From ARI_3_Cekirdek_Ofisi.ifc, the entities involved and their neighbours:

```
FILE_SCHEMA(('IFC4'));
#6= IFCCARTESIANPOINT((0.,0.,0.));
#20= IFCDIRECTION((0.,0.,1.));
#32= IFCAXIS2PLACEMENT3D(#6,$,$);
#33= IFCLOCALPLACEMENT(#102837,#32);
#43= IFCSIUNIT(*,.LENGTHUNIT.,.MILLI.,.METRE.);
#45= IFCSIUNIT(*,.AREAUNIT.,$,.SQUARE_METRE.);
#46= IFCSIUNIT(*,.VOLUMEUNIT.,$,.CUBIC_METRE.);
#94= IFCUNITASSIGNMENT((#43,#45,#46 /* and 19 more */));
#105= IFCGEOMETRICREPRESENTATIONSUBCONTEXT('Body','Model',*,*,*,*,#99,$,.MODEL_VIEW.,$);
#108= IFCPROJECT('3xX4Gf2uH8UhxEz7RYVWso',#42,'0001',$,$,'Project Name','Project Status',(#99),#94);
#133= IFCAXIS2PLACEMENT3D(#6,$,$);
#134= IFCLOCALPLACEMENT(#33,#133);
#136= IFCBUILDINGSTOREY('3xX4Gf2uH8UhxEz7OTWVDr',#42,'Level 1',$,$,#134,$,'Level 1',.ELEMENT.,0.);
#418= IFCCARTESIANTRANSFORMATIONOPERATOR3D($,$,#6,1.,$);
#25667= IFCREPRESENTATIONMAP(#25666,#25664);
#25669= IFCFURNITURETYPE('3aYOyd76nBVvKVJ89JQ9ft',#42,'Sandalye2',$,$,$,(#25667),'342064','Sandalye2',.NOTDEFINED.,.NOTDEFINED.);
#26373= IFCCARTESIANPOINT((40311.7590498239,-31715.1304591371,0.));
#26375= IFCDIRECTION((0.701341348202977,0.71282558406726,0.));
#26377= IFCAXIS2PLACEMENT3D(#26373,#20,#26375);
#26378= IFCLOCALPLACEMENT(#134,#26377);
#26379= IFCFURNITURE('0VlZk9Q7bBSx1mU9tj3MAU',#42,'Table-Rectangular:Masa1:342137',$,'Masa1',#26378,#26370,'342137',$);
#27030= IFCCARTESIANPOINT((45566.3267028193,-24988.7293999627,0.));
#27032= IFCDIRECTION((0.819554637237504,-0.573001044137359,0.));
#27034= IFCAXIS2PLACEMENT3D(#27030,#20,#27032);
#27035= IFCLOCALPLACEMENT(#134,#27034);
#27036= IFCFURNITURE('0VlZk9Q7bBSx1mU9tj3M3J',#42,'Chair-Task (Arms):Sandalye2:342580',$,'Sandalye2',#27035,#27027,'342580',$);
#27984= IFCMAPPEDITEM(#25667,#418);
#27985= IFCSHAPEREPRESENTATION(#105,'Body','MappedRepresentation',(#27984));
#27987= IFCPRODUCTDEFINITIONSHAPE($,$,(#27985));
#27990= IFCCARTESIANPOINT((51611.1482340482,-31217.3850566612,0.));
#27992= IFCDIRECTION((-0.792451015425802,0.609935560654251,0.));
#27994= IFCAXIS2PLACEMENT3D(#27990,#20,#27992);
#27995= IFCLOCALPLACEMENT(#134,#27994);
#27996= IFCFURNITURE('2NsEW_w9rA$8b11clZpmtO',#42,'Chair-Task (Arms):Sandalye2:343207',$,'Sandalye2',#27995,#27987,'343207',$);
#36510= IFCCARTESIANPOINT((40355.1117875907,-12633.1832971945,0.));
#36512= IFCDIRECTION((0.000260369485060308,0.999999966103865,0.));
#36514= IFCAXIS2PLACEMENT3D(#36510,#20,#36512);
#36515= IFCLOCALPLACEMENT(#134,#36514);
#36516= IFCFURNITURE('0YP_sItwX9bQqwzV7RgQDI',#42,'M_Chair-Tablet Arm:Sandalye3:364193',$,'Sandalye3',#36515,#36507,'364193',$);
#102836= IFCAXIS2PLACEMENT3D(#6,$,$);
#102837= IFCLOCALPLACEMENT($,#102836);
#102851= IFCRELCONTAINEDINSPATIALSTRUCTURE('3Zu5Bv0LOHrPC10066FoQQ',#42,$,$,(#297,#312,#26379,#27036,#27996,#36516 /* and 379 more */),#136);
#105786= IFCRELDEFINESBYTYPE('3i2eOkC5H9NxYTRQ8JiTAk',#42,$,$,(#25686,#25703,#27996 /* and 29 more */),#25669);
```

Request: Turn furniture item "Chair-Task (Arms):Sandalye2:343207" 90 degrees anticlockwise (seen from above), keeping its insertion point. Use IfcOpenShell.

```python
import ifcopenshell
import ifcopenshell.api.geometry
import ifcopenshell.util.placement

model = ifcopenshell.open("ARI_3_Cekirdek_Ofisi.ifc")

item = model.by_id(27996)
matrix = ifcopenshell.util.placement.get_local_placement(item.ObjectPlacement)
matrix = matrix @ ifcopenshell.util.placement.rotation(90, "Z")
ifcopenshell.api.geometry.edit_object_placement(model, product=item, matrix=matrix, is_si=False)

print(ifcopenshell.util.placement.get_local_placement(item.ObjectPlacement).round(3) + 0.0)

model.write("ARI_3_Cekirdek_Ofisi_updated.ifc")
```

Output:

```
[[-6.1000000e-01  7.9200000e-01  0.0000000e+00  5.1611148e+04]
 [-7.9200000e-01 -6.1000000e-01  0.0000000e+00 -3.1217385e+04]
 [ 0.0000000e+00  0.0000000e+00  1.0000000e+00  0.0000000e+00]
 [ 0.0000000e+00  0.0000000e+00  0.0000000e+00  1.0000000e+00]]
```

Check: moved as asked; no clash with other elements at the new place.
